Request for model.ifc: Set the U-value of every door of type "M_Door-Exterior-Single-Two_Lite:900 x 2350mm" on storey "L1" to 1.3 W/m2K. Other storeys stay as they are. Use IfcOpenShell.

First a look at what the model holds.

```python
import ifcopenshell
import ifcopenshell.util.element

model = ifcopenshell.open("model.ifc")
print(model.schema)
storey = next(s for s in model.by_type("IfcBuildingStorey") if s.Name == "L1")
doors = [e for e in ifcopenshell.util.element.get_decomposition(storey) if e.is_a("IfcDoor")]
seen = {}
for e in doors:
    element_type = ifcopenshell.util.element.get_type(e)
    key = (element_type.Name if element_type != e and element_type else None, ifcopenshell.util.element.get_pset(e, "Pset_DoorCommon", "ThermalTransmittance"))
    seen[key] = seen.get(key, 0) + 1
for (name, value), count in sorted(seen.items(), key=str):
    print(count, "x", name, "|", value)
```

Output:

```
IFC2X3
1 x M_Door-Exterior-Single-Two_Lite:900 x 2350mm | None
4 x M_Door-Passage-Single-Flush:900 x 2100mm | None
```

```python
import ifcopenshell
import ifcopenshell.api.pset
import ifcopenshell.util.element

model = ifcopenshell.open("model.ifc")

storey = next(s for s in model.by_type("IfcBuildingStorey") if s.Name == "L1")
doors = [e for e in ifcopenshell.util.element.get_decomposition(storey) if e.is_a("IfcDoor")]

count = 0
for e in doors:
    element_type = ifcopenshell.util.element.get_type(e)
    if element_type in (None, e) or element_type.Name != "M_Door-Exterior-Single-Two_Lite:900 x 2350mm":
        continue
    # add_pset returns the element's existing set when there is one.
    pset = ifcopenshell.api.pset.add_pset(model, product=e, name="Pset_DoorCommon")
    ifcopenshell.api.pset.edit_pset(model, pset=pset, properties={"ThermalTransmittance": 1.3})
    count += 1

print(count, "doors updated")

model.write("model_v2.ifc")
```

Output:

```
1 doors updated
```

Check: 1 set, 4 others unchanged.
